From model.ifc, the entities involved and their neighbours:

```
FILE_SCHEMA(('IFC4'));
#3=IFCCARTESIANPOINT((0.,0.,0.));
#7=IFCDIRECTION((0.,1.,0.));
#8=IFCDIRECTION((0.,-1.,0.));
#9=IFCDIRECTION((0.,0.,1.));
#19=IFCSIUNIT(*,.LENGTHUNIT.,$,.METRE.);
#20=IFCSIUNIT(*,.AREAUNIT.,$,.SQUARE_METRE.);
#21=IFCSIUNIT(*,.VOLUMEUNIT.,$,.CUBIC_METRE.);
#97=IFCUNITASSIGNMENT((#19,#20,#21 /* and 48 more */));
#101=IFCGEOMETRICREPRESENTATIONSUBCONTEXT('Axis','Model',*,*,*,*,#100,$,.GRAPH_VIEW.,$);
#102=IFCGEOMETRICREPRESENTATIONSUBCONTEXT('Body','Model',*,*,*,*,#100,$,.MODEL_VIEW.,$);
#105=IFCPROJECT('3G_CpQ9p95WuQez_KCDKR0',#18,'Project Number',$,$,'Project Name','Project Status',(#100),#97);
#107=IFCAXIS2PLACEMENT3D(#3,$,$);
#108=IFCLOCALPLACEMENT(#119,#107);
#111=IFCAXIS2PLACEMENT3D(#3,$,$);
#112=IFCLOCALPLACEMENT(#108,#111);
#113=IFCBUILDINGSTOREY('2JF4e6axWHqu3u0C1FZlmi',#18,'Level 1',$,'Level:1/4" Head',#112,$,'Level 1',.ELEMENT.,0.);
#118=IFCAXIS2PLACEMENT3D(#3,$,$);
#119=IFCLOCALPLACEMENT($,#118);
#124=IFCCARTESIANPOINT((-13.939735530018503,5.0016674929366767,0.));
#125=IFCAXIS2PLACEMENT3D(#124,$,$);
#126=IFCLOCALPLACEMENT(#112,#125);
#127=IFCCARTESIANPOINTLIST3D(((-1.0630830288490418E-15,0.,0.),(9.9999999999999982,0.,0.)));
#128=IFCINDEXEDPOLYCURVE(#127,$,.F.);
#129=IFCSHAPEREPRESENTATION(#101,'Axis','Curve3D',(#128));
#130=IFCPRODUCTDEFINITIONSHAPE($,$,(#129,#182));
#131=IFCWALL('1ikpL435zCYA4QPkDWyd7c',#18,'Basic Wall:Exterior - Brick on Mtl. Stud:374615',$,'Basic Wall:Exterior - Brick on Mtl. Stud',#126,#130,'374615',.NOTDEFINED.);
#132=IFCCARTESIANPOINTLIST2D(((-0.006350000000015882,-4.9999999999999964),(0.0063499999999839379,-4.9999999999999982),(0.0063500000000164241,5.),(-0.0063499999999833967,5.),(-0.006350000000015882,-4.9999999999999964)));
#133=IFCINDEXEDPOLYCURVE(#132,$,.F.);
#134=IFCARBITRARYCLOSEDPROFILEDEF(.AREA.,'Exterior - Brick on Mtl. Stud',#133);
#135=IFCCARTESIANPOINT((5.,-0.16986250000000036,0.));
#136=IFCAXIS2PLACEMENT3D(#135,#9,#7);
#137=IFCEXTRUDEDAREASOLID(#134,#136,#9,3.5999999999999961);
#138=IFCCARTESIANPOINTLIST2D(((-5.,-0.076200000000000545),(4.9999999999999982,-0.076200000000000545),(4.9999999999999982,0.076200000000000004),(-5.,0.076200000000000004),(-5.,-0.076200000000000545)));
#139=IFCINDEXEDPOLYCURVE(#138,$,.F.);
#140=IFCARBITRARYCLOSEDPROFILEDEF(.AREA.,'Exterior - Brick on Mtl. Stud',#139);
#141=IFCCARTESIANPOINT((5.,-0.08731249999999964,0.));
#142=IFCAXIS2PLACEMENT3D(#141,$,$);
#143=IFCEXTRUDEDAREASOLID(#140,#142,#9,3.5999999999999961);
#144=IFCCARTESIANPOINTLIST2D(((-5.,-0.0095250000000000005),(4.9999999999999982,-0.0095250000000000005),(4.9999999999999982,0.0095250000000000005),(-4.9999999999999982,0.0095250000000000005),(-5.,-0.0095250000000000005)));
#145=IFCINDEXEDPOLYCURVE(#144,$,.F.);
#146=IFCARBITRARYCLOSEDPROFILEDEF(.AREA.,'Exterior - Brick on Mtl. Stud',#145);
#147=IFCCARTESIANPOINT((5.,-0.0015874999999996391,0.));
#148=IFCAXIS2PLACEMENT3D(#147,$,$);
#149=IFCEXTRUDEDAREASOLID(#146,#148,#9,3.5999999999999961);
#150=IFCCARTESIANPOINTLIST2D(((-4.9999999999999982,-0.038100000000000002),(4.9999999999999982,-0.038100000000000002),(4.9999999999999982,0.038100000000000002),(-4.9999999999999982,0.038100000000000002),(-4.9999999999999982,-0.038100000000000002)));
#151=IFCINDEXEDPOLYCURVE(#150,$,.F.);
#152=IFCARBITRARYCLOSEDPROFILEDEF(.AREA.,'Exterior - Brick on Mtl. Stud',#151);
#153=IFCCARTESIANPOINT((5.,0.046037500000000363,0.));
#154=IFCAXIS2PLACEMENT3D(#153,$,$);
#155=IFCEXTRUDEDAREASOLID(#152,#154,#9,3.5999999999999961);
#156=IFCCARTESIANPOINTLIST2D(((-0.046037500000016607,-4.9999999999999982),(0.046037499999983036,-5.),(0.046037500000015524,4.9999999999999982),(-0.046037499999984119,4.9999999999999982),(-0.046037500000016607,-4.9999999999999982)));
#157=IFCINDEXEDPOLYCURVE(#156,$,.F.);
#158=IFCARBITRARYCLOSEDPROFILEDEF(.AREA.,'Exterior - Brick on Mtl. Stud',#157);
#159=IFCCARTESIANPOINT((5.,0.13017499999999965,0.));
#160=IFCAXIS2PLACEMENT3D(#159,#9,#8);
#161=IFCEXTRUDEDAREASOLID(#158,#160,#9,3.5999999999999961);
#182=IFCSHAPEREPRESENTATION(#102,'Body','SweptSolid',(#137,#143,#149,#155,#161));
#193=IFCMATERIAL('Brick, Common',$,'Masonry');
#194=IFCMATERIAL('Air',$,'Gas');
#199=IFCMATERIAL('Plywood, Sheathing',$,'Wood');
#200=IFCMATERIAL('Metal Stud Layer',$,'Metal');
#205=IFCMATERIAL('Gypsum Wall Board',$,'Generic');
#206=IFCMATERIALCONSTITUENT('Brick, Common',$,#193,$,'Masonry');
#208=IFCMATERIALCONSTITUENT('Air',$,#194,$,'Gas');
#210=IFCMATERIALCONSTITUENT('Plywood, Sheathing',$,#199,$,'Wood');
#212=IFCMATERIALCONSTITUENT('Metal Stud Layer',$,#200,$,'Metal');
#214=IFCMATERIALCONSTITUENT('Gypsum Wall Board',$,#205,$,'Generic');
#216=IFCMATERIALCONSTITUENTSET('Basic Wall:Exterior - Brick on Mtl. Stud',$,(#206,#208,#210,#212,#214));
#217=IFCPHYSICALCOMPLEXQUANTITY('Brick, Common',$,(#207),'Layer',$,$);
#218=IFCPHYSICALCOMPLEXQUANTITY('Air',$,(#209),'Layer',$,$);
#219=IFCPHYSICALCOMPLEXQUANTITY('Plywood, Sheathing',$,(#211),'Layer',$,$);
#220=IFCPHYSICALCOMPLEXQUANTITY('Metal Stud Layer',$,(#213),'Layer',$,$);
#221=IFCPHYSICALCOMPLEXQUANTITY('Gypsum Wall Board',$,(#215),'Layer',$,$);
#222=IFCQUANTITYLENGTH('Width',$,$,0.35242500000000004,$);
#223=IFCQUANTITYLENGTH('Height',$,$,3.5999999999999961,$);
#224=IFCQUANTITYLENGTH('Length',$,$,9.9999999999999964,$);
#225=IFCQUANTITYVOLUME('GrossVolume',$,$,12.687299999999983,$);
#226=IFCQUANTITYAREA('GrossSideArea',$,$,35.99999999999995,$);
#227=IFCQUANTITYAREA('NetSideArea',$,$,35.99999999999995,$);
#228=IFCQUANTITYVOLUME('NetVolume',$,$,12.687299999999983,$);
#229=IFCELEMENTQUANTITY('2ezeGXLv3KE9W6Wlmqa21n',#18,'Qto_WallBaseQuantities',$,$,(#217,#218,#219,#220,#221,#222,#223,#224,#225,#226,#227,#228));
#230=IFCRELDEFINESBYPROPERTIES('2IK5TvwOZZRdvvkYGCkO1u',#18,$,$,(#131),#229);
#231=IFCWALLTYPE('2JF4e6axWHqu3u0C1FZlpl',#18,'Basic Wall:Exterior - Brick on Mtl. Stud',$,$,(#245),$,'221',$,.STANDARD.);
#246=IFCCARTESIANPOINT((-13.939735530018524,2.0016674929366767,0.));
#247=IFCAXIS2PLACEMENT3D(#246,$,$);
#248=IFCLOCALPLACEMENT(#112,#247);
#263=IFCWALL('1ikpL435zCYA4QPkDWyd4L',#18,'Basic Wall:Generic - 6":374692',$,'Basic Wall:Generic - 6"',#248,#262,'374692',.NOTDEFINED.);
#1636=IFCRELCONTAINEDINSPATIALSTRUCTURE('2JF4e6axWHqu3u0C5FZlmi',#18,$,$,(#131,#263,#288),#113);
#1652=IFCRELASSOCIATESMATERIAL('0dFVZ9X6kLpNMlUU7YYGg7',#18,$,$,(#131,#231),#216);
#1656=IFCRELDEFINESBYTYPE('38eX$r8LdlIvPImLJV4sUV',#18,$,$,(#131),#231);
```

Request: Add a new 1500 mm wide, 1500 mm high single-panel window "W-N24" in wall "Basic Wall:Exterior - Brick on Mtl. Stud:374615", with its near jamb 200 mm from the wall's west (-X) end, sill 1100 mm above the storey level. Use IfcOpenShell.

```python
import numpy as np
import ifcopenshell
import ifcopenshell.api.feature
import ifcopenshell.api.geometry
import ifcopenshell.api.pset
import ifcopenshell.api.root
import ifcopenshell.api.spatial
import ifcopenshell.geom
import ifcopenshell.util.element
import ifcopenshell.util.placement
import ifcopenshell.util.representation
import ifcopenshell.util.shape
import ifcopenshell.util.unit

model = ifcopenshell.open("model.ifc")
unit_scale = ifcopenshell.util.unit.calculate_unit_scale(model)
area_scale = ifcopenshell.util.unit.calculate_unit_scale(model, "AREAUNIT")
volume_scale = ifcopenshell.util.unit.calculate_unit_scale(model, "VOLUMEUNIT")
settings = ifcopenshell.geom.settings()


def volume(element):
    """Net volume in cubic metres, openings subtracted."""
    shape = ifcopenshell.geom.create_shape(settings, element)
    return ifcopenshell.util.shape.get_volume(shape.geometry)


wall = model.by_guid("1ikpL435zCYA4QPkDWyd7c")
storey = ifcopenshell.util.element.get_container(wall, ifc_class="IfcBuildingStorey")
context = ifcopenshell.util.representation.get_context(model, "Model", "Body", "MODEL_VIEW")
before = volume(wall)

width, height, from_end, sill = 1.5, 1.5, 0.2, 1.1  # metres

# The wall runs along its own X axis, and the end named is its -X end.
wall_shape = ifcopenshell.geom.create_shape(settings, wall)
x, y, z = ifcopenshell.util.shape.get_vertices(wall_shape.geometry).T
start = x.min() + from_end
face, thickness = float(y.min()), float(y.max() - y.min())
wall_matrix = ifcopenshell.util.placement.get_local_placement(wall.ObjectPlacement)
level = ifcopenshell.util.placement.get_local_placement(storey.ObjectPlacement)[2, 3]


def in_wall(x, y):
    """Placement at x, y metres in the wall's axes, at sill height."""
    matrix = wall_matrix.copy()
    matrix[:, 3] = wall_matrix @ np.array([x / unit_scale, y / unit_scale, 0.0, 1.0])
    matrix[2, 3] = level + sill / unit_scale
    return matrix


# Opening: a box that overshoots both wall faces by 50 mm.
opening = ifcopenshell.api.root.create_entity(model, ifc_class="IfcOpeningElement", predefined_type="OPENING")
box = ifcopenshell.api.geometry.add_wall_representation(
    model, context=context, length=width, height=height, thickness=thickness + 0.1
)
ifcopenshell.api.geometry.assign_representation(model, product=opening, representation=box)
ifcopenshell.api.geometry.edit_object_placement(model, product=opening, matrix=in_wall(start, face - 0.05), is_si=False)
ifcopenshell.api.feature.add_feature(model, feature=opening, element=wall)

window = ifcopenshell.api.root.create_entity(model, ifc_class="IfcWindow", name="W-N24", predefined_type="WINDOW")
window.OverallWidth, window.OverallHeight = width / unit_scale, height / unit_scale
window.PartitioningType = "SINGLE_PANEL"
body = ifcopenshell.api.geometry.add_window_representation(
    model,
    context=context,
    overall_width=window.OverallWidth,
    overall_height=window.OverallHeight,
    partition_type="SINGLE_PANEL",
)
ifcopenshell.api.geometry.assign_representation(model, product=window, representation=body)
ifcopenshell.api.spatial.assign_container(model, products=[window], relating_structure=storey)
ifcopenshell.api.feature.add_filling(model, opening=opening, element=window)

# Centre the window in the wall's thickness.
ifcopenshell.api.geometry.edit_object_placement(model, product=window, matrix=in_wall(start, face), is_si=False)
window_shape = ifcopenshell.geom.create_shape(settings, window)
depth = ifcopenshell.util.shape.get_vertices(window_shape.geometry)[:, 1]
offset = face + thickness / 2 - (depth.min() + depth.max()) / 2
ifcopenshell.api.geometry.edit_object_placement(model, product=window, matrix=in_wall(start, offset), is_si=False)

after = volume(wall)

# Update the wall's stored quantities.
qto = model.by_id(ifcopenshell.util.element.get_pset(wall, "Qto_WallBaseQuantities", should_inherit=False)["id"])
ifcopenshell.api.pset.edit_qto(model, qto=qto, properties={
    "NetSideArea": after / thickness / area_scale,
    "NetVolume": after / volume_scale,
})

print(f"wall volume {before:.3f} -> {after:.3f} m3")

model.write("model-out.ifc")
```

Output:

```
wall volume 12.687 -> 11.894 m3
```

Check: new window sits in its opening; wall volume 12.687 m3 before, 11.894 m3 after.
